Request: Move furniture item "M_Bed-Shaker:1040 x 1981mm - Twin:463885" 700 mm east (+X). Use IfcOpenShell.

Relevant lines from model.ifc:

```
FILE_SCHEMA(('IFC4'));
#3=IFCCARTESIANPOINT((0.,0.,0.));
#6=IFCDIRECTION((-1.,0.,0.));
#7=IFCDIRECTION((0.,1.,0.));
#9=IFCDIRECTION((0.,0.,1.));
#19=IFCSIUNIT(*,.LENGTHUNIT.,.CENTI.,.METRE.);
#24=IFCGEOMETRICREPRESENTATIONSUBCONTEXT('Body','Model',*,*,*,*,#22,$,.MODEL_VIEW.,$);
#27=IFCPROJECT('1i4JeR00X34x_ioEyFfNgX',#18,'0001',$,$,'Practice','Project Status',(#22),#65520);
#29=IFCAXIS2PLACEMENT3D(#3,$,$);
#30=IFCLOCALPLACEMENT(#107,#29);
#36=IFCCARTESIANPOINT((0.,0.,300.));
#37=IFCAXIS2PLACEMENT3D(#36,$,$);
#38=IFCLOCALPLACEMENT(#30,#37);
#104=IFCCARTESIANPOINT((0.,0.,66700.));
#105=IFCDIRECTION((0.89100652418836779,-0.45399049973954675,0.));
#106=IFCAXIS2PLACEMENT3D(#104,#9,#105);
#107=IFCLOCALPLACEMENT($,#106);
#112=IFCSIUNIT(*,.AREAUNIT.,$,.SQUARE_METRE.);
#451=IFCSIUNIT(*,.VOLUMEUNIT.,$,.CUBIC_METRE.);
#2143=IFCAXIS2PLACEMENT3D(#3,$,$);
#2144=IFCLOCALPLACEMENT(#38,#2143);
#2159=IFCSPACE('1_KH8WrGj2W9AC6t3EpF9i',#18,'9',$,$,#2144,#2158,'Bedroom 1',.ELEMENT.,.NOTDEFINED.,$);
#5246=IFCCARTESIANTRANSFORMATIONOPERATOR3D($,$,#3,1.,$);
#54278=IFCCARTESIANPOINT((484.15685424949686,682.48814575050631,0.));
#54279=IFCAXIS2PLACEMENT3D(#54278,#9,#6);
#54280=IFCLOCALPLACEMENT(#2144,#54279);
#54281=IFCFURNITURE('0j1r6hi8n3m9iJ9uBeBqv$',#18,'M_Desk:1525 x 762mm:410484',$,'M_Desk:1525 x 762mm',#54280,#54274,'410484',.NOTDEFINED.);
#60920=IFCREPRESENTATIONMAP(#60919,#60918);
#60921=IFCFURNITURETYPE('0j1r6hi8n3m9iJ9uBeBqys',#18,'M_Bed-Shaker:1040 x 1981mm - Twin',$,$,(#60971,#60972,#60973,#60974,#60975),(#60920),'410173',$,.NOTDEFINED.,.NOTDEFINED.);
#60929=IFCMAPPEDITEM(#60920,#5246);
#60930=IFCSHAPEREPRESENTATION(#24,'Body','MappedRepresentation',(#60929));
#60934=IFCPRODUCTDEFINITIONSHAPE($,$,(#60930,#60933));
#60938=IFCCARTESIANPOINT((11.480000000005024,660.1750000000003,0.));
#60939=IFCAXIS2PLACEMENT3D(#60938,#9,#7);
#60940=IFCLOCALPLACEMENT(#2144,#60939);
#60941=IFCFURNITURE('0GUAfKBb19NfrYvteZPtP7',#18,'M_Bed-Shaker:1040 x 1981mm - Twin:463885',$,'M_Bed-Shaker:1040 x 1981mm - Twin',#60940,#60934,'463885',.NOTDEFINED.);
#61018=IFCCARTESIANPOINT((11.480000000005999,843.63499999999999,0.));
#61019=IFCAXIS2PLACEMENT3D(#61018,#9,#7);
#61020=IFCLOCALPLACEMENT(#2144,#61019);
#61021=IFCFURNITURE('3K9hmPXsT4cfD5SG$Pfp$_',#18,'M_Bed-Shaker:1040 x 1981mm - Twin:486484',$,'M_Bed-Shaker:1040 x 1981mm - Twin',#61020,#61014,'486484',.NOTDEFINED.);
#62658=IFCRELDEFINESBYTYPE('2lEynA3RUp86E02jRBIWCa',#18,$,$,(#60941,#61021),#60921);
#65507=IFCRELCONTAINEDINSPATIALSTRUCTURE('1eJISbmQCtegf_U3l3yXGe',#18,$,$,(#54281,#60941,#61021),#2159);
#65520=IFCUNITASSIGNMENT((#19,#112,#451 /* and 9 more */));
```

```python
import ifcopenshell
import ifcopenshell.api.geometry
import ifcopenshell.util.placement
import ifcopenshell.util.unit

model = ifcopenshell.open("model.ifc")
unit_scale = ifcopenshell.util.unit.calculate_unit_scale(model)

item = model.by_guid("0GUAfKBb19NfrYvteZPtP7")
matrix = ifcopenshell.util.placement.get_local_placement(item.ObjectPlacement)
matrix[0, 3] += 0.7 / unit_scale
ifcopenshell.api.geometry.edit_object_placement(model, product=item, matrix=matrix, is_si=False)

print(ifcopenshell.util.placement.get_local_placement(item.ObjectPlacement).round(3) + 0.0)

model.write("model_v2.ifc")
```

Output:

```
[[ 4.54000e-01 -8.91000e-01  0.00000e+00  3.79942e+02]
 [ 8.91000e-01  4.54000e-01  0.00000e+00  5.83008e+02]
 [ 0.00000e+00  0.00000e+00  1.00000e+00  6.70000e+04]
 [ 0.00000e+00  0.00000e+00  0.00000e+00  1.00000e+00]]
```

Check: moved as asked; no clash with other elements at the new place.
